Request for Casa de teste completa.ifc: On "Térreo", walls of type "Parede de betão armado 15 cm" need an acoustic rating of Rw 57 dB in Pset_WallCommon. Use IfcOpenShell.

First a look at what the model holds.

```python
import ifcopenshell
import ifcopenshell.util.element

model = ifcopenshell.open("Casa de teste completa.ifc")
print(model.schema)
storey = next(s for s in model.by_type("IfcBuildingStorey") if s.Name == "Térreo")
walls = [e for e in ifcopenshell.util.element.get_decomposition(storey) if e.is_a("IfcWall")]
seen = {}
for e in walls:
    element_type = ifcopenshell.util.element.get_type(e)
    key = (element_type.Name if element_type != e and element_type else None, ifcopenshell.util.element.get_pset(e, "Pset_WallCommon", "AcousticRating"))
    seen[key] = seen.get(key, 0) + 1
for (name, value), count in sorted(seen.items(), key=str):
    print(count, "x", name, "|", value)
```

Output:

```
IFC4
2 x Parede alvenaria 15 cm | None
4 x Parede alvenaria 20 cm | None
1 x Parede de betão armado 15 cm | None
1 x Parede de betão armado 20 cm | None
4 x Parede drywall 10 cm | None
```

```python
import ifcopenshell
import ifcopenshell.api.pset
import ifcopenshell.util.element

model = ifcopenshell.open("Casa de teste completa.ifc")

storey = next(s for s in model.by_type("IfcBuildingStorey") if s.Name == "Térreo")
walls = [e for e in ifcopenshell.util.element.get_decomposition(storey) if e.is_a("IfcWall")]

count = 0
for e in walls:
    element_type = ifcopenshell.util.element.get_type(e)
    if element_type in (None, e) or element_type.Name != "Parede de betão armado 15 cm":
        continue
    # add_pset returns the element's existing set when there is one.
    pset = ifcopenshell.api.pset.add_pset(model, product=e, name="Pset_WallCommon")
    ifcopenshell.api.pset.edit_pset(model, pset=pset, properties={"AcousticRating": "Rw 57 dB"})
    count += 1

print(count, "walls updated")

model.write("Casa de teste completa_v2.ifc")
```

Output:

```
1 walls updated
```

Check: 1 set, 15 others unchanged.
